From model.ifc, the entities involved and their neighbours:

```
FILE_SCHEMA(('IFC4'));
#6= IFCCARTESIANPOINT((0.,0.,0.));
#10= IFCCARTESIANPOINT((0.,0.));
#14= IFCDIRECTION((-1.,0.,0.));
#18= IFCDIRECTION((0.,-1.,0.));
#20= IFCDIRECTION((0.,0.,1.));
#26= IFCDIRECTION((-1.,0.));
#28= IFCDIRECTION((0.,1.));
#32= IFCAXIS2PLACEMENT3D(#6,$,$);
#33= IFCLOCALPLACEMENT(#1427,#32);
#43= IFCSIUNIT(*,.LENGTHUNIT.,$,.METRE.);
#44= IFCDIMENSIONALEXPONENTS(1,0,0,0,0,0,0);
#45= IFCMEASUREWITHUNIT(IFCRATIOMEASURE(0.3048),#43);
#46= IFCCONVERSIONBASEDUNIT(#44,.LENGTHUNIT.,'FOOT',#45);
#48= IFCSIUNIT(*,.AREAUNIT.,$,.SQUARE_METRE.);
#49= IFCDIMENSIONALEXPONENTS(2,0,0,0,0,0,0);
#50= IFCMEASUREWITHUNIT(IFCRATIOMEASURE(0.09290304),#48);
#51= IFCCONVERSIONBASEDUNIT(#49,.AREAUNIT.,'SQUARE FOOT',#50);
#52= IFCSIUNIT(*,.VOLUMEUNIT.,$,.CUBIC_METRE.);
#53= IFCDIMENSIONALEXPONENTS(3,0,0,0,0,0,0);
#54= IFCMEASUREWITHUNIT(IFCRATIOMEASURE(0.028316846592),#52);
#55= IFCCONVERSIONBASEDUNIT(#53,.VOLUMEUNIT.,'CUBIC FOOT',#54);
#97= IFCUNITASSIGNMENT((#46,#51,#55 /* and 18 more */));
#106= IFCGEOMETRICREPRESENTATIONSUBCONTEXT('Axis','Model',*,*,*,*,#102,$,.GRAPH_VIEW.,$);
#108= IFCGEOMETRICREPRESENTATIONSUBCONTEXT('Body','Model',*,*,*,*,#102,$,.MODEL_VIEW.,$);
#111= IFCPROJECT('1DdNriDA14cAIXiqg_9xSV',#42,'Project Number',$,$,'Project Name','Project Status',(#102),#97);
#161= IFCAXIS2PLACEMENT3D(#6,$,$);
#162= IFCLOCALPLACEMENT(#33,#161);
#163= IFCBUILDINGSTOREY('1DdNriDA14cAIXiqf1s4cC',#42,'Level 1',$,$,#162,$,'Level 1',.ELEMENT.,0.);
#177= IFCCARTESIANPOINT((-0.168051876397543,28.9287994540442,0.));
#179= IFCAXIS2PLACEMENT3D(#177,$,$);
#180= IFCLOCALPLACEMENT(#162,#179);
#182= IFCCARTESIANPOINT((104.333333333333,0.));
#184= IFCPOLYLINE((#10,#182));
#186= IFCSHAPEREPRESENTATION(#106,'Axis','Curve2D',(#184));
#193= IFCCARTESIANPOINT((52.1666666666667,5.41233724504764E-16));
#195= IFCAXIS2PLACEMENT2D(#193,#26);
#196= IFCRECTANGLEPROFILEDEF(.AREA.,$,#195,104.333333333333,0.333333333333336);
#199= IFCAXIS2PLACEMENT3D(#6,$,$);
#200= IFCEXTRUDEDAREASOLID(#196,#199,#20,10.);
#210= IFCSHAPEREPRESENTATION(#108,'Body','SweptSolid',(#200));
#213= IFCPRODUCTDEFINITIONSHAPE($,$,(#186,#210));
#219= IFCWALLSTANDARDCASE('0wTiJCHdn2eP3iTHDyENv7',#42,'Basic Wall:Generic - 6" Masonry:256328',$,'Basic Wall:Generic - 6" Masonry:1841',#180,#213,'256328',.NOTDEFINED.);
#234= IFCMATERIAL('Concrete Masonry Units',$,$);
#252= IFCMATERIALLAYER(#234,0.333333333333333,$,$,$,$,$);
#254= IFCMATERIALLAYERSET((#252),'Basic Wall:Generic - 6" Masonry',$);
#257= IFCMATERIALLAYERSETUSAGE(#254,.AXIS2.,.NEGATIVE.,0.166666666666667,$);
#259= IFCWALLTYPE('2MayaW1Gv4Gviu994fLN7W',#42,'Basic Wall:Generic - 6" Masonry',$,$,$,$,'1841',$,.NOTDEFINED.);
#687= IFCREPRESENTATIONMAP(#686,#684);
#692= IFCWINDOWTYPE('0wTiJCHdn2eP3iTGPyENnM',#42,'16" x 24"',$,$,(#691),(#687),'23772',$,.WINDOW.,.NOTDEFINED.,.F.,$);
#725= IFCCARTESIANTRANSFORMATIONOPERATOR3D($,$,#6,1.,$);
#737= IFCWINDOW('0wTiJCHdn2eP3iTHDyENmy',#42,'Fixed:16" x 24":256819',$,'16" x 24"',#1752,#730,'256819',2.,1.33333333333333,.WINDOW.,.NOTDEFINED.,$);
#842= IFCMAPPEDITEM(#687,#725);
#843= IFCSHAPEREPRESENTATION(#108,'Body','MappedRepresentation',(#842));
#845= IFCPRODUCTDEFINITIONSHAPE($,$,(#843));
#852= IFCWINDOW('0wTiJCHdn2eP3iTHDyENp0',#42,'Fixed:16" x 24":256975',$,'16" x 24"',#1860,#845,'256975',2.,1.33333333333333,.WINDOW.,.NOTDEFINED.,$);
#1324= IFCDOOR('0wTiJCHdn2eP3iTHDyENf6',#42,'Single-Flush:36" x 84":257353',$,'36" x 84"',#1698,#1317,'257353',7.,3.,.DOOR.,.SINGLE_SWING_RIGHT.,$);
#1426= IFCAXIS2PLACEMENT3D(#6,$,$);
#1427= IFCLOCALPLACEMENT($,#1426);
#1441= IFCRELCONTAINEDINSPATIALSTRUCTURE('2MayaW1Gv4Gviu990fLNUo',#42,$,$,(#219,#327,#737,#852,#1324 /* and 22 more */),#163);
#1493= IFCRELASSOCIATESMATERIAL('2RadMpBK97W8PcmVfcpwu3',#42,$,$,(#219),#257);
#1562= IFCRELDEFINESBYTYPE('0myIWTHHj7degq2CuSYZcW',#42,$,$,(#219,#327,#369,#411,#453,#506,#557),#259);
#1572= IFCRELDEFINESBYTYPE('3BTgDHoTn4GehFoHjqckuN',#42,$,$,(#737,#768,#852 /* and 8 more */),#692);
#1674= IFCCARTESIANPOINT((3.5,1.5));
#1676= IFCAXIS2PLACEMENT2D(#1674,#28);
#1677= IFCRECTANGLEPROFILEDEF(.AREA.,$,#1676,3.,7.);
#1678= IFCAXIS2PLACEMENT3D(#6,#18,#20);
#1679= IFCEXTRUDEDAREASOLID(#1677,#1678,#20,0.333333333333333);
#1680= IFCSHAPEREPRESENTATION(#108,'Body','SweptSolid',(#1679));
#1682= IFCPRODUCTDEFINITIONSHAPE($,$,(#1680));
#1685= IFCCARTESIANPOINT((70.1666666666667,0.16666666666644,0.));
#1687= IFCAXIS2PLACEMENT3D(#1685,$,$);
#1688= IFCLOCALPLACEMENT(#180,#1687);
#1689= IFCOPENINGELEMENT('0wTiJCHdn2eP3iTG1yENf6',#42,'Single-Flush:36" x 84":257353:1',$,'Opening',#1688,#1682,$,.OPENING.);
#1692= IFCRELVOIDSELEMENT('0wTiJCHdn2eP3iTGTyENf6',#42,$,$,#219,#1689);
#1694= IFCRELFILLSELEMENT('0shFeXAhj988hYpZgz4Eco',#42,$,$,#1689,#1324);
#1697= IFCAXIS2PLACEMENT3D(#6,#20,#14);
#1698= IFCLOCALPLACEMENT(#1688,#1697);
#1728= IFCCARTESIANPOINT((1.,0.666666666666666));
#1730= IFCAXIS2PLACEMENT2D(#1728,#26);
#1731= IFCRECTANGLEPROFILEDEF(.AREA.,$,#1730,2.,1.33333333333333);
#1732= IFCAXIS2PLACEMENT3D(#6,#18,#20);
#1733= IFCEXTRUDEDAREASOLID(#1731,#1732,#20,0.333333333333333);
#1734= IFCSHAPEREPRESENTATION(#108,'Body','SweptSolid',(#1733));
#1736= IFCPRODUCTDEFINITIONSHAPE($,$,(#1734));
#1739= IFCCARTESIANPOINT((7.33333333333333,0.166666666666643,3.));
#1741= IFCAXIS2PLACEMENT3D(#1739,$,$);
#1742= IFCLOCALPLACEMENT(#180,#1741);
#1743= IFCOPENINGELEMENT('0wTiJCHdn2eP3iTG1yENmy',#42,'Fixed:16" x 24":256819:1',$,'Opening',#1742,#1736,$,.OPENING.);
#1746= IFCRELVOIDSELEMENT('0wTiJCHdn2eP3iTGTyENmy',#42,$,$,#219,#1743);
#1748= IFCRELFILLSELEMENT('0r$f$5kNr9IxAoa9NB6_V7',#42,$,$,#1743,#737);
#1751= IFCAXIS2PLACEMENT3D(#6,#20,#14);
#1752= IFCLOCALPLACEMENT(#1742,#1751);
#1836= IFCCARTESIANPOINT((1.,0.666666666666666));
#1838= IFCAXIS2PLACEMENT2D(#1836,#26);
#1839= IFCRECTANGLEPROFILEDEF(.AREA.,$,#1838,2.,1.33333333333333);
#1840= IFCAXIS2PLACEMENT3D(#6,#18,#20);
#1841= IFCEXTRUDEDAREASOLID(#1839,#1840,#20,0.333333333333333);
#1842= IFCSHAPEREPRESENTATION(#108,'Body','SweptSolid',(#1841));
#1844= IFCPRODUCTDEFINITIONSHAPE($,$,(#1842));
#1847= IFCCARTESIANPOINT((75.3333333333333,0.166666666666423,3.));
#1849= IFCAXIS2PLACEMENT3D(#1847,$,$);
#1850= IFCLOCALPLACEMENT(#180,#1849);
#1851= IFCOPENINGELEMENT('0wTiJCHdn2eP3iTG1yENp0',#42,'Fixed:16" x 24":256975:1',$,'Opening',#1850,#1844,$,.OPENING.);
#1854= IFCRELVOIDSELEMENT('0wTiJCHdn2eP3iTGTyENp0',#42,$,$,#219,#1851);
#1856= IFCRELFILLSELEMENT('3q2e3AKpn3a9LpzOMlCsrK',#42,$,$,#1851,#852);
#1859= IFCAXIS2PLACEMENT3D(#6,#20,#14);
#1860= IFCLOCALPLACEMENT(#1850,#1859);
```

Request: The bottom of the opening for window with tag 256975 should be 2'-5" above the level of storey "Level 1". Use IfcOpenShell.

```python
import numpy as np
import ifcopenshell
import ifcopenshell.api.geometry
import ifcopenshell.geom
import ifcopenshell.util.element
import ifcopenshell.util.placement
import ifcopenshell.util.shape
import ifcopenshell.util.unit

model = ifcopenshell.open("model.ifc")
unit_scale = ifcopenshell.util.unit.calculate_unit_scale(model)

window = model.by_guid("0wTiJCHdn2eP3iTHDyENp0")
opening = window.FillsVoids[0].RelatingOpeningElement
storey = ifcopenshell.util.element.get_container(window, ifc_class="IfcBuildingStorey")
level = ifcopenshell.util.placement.get_local_placement(storey.ObjectPlacement)[2, 3]

# The opening's origin need not be at the sill, so measure its lowest point.
shape = ifcopenshell.geom.create_shape(ifcopenshell.geom.settings(), opening)
bottom = ifcopenshell.util.shape.get_shape_bottom_elevation(shape, shape.geometry) / unit_scale
dz = level + 29 * 0.0254 / unit_scale - bottom

shift = np.array([0.0, 0.0, dz])
# The window is placed relative to its opening, so it follows when the opening moves.
matrix = ifcopenshell.util.placement.get_local_placement(opening.ObjectPlacement)
matrix[:3, 3] += shift
ifcopenshell.api.geometry.edit_object_placement(
    model, product=opening, matrix=matrix, is_si=False, should_transform_children=True
)

print(f"moved by {dz * unit_scale:+.3f} m")

model.write("model_rev.ifc")
```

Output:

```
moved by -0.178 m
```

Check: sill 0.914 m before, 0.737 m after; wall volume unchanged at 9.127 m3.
